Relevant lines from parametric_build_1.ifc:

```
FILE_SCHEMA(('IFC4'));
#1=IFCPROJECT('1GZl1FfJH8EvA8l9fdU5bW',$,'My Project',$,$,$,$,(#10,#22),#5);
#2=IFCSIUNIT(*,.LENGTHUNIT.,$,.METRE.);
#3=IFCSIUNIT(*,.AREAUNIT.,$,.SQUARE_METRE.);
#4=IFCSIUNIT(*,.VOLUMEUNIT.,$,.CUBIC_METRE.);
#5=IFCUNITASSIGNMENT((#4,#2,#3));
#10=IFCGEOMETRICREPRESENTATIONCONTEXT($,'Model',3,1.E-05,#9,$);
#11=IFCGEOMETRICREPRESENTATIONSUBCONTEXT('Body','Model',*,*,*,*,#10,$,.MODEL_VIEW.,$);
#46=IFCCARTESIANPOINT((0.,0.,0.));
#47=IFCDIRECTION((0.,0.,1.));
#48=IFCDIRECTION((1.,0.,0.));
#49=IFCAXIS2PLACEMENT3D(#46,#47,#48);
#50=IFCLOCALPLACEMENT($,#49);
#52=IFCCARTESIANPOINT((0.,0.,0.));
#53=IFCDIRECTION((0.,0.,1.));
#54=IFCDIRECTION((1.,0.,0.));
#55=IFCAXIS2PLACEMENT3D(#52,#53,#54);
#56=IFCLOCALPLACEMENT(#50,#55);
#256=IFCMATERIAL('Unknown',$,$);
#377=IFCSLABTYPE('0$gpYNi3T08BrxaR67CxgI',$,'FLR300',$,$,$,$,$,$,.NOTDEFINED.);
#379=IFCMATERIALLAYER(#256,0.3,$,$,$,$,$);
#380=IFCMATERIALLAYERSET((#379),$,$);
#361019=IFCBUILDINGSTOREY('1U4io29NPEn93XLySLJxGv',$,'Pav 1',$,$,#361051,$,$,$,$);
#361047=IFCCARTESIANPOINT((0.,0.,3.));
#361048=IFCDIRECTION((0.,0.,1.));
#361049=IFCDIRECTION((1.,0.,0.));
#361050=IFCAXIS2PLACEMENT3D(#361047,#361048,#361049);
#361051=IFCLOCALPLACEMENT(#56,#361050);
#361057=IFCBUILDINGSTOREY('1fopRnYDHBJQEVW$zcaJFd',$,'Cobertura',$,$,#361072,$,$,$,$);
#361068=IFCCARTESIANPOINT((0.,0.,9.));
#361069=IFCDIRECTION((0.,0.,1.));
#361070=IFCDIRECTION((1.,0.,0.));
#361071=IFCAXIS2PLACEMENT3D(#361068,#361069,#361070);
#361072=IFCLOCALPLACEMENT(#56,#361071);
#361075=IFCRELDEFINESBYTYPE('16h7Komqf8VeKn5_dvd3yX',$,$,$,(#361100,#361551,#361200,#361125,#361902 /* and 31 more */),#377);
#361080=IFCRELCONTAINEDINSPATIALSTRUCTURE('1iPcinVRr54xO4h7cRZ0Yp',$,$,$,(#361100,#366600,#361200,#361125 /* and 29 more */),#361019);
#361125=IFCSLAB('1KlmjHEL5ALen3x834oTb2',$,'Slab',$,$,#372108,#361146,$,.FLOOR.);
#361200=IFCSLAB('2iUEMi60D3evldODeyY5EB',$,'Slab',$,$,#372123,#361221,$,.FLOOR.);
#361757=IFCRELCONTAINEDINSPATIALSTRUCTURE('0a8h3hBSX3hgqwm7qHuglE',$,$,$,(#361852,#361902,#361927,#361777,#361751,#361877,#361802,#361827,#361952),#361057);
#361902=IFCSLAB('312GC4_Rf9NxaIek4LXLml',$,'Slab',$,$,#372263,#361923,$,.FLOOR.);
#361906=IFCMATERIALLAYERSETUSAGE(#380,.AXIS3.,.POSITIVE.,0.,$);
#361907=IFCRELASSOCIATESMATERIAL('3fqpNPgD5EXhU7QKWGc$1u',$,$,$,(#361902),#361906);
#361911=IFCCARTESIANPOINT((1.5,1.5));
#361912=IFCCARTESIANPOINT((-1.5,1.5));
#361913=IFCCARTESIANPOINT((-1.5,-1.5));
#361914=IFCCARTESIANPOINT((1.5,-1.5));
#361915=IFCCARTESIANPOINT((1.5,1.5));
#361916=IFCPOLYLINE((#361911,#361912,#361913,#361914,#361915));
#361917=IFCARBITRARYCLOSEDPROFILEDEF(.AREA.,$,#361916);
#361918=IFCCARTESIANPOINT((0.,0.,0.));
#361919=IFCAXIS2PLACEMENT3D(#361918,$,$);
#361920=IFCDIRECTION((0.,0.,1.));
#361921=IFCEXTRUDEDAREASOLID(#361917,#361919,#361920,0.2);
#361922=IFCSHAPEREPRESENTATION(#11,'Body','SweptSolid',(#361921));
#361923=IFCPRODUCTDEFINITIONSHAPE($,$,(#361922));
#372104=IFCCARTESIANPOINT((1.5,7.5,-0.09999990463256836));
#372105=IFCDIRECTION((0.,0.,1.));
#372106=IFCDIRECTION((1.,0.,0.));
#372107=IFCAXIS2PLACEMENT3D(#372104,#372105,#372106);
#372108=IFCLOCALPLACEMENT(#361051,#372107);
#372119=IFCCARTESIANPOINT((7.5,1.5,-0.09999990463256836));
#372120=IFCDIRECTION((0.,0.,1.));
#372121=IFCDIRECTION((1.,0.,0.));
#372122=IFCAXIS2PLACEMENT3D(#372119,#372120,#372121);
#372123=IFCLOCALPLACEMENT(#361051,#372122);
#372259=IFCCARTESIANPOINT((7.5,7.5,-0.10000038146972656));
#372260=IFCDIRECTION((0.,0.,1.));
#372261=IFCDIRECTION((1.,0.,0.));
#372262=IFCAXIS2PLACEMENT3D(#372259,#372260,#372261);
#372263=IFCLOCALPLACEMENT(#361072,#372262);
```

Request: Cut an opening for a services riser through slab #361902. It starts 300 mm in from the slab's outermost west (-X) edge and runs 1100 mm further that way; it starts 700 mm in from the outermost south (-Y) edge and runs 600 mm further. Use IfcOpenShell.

```python
import numpy as np
import ifcopenshell
import ifcopenshell.api.feature
import ifcopenshell.api.geometry
import ifcopenshell.api.root
import ifcopenshell.geom
import ifcopenshell.util.placement
import ifcopenshell.util.representation
import ifcopenshell.util.shape
import ifcopenshell.util.unit

model = ifcopenshell.open("parametric_build_1.ifc")
unit_scale = ifcopenshell.util.unit.calculate_unit_scale(model)
settings = ifcopenshell.geom.settings()


def volume(element):
    """Net volume in cubic metres, openings subtracted."""
    shape = ifcopenshell.geom.create_shape(settings, element)
    return ifcopenshell.util.shape.get_volume(shape.geometry)


slab = model.by_guid("312GC4_Rf9NxaIek4LXLml")
before = volume(slab)

# Extent in the slab's own axes, in metres. The edges named are its -X and -Y sides.
slab_shape = ifcopenshell.geom.create_shape(settings, slab)
vertices = ifcopenshell.util.shape.get_vertices(slab_shape.geometry)
x_min, y_min, bottom = vertices.min(axis=0)
top = vertices[:, 2].max()

opening = ifcopenshell.api.root.create_entity(model, ifc_class="IfcOpeningElement", name="Services riser opening", predefined_type="OPENING")
context = ifcopenshell.util.representation.get_context(model, "Model", "Body", "MODEL_VIEW")
width, depth = 1.1, 0.6
outline = [(0.0, 0.0), (width, 0.0), (width, depth), (0.0, depth), (0.0, 0.0)]
# Overshoot both faces by 50 mm so the cut is clean.
shape = ifcopenshell.api.geometry.add_slab_representation(
    model, context=context, depth=top - bottom + 0.1, polyline=outline
)
ifcopenshell.api.geometry.assign_representation(model, product=opening, representation=shape)

matrix = ifcopenshell.util.placement.get_local_placement(slab.ObjectPlacement)
matrix[:, 3] = matrix @ np.append(np.array([x_min + 0.3, y_min + 0.7, bottom - 0.05]) / unit_scale, 1.0)
ifcopenshell.api.geometry.edit_object_placement(model, product=opening, matrix=matrix, is_si=False)
ifcopenshell.api.feature.add_feature(model, feature=opening, element=slab)

after = volume(slab)

print(f"slab volume {before:.3f} -> {after:.3f} m3")

model.write("parametric_build_1-out.ifc")
```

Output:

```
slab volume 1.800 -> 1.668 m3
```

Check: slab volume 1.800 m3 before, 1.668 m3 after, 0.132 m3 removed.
